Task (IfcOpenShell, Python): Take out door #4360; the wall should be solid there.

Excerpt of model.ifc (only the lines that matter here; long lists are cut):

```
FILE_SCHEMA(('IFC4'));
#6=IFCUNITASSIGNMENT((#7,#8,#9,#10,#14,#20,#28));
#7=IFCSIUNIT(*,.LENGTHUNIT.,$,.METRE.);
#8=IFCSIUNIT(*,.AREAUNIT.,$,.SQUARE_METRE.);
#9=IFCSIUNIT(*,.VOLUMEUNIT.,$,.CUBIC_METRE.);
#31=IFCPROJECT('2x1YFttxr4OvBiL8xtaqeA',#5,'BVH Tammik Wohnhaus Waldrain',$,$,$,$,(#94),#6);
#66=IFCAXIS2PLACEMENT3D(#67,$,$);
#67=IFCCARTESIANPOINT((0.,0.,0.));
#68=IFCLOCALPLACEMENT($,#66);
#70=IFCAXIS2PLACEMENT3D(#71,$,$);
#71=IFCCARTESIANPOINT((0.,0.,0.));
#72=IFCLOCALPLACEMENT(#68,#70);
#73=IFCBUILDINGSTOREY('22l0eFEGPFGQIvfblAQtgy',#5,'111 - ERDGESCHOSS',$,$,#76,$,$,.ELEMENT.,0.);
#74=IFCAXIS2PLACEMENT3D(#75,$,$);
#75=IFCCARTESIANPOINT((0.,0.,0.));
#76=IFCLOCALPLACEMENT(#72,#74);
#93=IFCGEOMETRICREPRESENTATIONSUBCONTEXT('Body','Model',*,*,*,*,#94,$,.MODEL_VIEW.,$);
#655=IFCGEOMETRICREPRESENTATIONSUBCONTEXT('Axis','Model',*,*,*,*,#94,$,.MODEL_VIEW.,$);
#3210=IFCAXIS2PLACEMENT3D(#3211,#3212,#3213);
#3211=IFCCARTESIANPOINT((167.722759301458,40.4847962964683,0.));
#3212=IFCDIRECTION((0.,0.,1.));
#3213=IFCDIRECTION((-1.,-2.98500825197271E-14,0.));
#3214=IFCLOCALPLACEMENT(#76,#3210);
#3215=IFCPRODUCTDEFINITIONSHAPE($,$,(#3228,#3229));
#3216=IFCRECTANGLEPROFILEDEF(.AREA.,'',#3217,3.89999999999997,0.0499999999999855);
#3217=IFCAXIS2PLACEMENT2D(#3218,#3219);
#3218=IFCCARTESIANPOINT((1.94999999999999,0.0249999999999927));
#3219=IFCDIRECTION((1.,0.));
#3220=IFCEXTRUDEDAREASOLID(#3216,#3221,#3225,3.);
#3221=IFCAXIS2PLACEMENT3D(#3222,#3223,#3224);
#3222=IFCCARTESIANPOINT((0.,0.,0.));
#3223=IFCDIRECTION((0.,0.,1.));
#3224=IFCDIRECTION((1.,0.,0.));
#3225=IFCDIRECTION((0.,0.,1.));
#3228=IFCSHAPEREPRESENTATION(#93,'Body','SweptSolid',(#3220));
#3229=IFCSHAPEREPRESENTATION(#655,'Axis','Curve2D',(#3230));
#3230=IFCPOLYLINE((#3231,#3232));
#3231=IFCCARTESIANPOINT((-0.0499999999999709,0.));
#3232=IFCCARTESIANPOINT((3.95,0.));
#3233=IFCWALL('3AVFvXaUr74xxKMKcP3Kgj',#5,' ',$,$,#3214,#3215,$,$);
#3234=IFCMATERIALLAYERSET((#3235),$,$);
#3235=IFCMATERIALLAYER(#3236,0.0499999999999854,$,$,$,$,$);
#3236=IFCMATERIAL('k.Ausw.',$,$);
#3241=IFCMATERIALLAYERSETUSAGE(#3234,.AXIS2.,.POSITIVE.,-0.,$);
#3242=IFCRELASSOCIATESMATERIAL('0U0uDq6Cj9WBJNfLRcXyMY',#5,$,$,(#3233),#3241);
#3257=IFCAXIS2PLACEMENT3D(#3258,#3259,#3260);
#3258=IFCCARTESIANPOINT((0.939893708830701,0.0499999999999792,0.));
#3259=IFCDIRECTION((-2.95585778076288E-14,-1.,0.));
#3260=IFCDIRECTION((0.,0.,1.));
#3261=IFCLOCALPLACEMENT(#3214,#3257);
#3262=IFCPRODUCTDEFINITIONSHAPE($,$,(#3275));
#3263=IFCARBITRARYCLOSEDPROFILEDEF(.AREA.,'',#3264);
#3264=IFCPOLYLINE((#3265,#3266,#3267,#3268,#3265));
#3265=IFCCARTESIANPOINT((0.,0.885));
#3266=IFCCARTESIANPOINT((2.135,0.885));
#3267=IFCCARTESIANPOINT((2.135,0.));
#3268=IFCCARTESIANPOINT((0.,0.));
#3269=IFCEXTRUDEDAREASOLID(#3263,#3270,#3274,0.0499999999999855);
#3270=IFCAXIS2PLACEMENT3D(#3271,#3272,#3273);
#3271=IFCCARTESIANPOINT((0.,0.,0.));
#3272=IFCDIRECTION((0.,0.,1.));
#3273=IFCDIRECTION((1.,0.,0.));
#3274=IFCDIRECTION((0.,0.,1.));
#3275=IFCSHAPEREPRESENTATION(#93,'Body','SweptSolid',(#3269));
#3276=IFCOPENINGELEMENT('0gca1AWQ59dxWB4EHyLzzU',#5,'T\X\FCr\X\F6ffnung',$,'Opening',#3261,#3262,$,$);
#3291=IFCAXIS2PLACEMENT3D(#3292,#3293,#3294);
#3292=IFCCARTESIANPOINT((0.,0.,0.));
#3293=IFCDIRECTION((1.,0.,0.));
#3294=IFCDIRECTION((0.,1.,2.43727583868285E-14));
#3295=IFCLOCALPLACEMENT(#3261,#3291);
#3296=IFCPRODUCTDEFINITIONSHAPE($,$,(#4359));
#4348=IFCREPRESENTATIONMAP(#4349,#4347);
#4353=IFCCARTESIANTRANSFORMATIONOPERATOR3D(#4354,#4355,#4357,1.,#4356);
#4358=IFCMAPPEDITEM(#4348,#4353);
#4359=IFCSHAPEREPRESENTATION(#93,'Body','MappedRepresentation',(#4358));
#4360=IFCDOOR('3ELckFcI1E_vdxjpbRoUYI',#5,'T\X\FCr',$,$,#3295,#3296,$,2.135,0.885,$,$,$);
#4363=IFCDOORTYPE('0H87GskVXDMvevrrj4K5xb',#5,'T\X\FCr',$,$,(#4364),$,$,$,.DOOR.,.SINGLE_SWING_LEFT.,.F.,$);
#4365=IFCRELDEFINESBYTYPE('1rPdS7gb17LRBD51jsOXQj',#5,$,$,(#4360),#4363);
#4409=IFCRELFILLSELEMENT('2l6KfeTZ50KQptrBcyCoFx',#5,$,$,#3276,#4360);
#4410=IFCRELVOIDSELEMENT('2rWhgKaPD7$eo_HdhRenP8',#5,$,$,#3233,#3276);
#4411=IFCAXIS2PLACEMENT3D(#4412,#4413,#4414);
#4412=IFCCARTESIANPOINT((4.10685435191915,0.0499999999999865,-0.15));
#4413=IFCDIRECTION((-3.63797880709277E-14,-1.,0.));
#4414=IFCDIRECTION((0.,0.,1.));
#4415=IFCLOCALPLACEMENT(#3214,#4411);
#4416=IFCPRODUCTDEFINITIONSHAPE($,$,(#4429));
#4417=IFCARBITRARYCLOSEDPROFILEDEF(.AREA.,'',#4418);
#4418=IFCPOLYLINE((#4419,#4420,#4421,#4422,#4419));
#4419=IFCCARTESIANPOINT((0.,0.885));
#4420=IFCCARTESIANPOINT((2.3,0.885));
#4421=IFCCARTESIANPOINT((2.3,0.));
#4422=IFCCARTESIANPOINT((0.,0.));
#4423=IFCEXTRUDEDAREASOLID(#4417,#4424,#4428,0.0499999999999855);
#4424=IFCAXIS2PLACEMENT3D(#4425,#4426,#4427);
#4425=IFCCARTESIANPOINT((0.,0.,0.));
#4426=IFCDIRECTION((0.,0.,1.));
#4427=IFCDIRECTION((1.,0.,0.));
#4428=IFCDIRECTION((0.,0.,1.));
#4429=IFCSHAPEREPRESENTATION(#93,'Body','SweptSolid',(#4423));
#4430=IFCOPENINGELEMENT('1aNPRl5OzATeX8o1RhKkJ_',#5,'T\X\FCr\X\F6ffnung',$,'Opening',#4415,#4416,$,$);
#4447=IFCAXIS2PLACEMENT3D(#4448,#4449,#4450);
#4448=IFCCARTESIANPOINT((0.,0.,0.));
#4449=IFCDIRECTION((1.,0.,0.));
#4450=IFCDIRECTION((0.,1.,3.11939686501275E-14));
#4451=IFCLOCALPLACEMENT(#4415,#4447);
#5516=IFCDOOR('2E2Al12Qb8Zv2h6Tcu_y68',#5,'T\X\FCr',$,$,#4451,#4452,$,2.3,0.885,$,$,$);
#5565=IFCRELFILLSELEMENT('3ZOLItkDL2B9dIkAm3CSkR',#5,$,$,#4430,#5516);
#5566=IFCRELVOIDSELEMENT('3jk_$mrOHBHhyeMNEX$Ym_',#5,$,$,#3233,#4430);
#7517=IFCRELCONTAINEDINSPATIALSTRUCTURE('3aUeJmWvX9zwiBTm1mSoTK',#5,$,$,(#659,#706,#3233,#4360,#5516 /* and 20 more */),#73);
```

```python
import ifcopenshell
import ifcopenshell.api.feature
import ifcopenshell.api.root
import ifcopenshell.geom
import ifcopenshell.util.shape

model = ifcopenshell.open("model.ifc")
settings = ifcopenshell.geom.settings()


def volume(element):
    """Net volume in cubic metres, openings subtracted."""
    shape = ifcopenshell.geom.create_shape(settings, element)
    return ifcopenshell.util.shape.get_volume(shape.geometry)


door = model.by_id(4360)
opening = door.FillsVoids[0].RelatingOpeningElement
wall = opening.VoidsElements[0].RelatingBuildingElement
before = volume(wall)

ifcopenshell.api.root.remove_product(model, product=door)
ifcopenshell.api.feature.remove_feature(model, feature=opening)

after = volume(wall)

print(f"wall volume {before:.3f} -> {after:.3f} m3")

model.write("model_updated.ifc")
```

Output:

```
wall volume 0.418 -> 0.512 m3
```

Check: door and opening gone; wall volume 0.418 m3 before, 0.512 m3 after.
